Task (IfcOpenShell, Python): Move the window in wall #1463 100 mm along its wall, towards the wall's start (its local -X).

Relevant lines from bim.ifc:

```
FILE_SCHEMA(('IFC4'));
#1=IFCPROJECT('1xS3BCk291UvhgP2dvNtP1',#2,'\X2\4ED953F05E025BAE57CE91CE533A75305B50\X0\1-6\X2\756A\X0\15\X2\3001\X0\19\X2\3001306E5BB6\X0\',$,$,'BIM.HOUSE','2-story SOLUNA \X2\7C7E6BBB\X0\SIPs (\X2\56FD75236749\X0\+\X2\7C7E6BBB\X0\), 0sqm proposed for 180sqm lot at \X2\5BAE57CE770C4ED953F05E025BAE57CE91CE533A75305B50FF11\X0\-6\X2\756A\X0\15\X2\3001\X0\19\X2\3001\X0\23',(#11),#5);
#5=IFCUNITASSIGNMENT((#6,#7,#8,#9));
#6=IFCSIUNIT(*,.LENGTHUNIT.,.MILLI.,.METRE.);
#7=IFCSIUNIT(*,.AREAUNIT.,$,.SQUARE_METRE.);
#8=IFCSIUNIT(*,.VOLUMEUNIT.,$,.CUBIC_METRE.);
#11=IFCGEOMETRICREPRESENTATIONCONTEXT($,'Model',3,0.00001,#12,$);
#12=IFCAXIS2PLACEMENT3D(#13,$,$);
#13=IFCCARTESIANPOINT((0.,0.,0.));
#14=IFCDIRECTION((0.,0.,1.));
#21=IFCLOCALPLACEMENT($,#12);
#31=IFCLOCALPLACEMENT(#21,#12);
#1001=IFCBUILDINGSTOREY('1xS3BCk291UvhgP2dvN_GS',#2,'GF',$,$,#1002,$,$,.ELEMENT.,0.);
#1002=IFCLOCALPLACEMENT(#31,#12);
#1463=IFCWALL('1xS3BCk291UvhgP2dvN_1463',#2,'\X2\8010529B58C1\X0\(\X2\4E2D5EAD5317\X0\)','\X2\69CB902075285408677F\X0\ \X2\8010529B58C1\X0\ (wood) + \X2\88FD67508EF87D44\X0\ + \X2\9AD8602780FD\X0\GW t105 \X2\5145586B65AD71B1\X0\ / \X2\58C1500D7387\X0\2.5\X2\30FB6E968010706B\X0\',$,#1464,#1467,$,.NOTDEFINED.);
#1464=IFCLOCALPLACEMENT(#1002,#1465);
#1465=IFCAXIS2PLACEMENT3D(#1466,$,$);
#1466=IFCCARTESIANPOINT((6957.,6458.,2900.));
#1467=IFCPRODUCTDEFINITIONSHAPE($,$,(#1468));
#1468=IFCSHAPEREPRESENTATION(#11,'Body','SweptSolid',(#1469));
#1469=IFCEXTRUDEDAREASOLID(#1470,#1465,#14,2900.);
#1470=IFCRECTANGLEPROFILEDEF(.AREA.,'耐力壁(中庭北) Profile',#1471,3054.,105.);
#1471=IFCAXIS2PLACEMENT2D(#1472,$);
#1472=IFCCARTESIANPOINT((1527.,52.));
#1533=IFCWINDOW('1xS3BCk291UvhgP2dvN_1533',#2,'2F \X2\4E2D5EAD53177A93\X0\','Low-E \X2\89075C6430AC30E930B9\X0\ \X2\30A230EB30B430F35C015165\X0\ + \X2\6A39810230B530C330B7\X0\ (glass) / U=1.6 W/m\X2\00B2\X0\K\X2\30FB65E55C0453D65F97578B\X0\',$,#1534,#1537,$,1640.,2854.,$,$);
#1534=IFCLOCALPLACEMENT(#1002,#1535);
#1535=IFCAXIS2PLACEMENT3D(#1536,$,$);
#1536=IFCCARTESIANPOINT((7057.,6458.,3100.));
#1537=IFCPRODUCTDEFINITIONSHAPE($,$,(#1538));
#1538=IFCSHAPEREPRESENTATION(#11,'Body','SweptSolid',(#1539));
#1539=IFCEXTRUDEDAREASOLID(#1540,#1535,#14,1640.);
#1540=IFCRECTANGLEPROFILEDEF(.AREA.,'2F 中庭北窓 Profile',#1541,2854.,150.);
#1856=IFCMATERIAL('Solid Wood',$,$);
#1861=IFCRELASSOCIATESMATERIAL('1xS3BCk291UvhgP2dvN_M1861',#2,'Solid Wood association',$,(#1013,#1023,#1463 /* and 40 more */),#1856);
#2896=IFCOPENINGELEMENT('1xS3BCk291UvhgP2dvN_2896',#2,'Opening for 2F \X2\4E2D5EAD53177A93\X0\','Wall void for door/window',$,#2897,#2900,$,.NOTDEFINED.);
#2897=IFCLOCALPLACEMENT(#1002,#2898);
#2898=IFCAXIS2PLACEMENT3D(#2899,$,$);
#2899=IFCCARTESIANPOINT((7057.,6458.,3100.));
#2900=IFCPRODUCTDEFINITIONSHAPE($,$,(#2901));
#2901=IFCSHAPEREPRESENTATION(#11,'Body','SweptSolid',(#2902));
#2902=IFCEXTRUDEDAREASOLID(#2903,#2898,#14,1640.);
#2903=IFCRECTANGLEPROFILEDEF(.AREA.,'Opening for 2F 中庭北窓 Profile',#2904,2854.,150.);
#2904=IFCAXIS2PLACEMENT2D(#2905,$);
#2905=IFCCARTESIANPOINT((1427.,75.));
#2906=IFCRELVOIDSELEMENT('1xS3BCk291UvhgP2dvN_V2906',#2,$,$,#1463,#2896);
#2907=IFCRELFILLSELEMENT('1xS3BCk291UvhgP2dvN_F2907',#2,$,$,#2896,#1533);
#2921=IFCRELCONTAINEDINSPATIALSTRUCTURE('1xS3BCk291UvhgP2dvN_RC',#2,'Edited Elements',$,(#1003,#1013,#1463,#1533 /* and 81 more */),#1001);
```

```python
import ifcopenshell
import ifcopenshell.api.geometry
import ifcopenshell.util.placement

model = ifcopenshell.open("bim.ifc")

window = model.by_id(1533)
opening = window.FillsVoids[0].RelatingOpeningElement
wall = opening.VoidsElements[0].RelatingBuildingElement

wall_matrix = ifcopenshell.util.placement.get_local_placement(wall.ObjectPlacement)
shift = wall_matrix[:3, 0] * -100.0
before = ifcopenshell.util.placement.get_local_placement(window.ObjectPlacement)[:3, 3].copy()

# The window is not placed relative to its opening, so move both.
for product in (opening, window):
    matrix = ifcopenshell.util.placement.get_local_placement(product.ObjectPlacement)
    matrix[:3, 3] += shift
    ifcopenshell.api.geometry.edit_object_placement(model, product=product, matrix=matrix, is_si=False)

after = ifcopenshell.util.placement.get_local_placement(window.ObjectPlacement)[:3, 3]
print("window moved by", (after - before).round(3) + 0.0)

model.write("bim_updated.ifc")
```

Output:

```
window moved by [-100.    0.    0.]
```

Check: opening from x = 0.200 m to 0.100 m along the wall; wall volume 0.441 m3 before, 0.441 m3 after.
